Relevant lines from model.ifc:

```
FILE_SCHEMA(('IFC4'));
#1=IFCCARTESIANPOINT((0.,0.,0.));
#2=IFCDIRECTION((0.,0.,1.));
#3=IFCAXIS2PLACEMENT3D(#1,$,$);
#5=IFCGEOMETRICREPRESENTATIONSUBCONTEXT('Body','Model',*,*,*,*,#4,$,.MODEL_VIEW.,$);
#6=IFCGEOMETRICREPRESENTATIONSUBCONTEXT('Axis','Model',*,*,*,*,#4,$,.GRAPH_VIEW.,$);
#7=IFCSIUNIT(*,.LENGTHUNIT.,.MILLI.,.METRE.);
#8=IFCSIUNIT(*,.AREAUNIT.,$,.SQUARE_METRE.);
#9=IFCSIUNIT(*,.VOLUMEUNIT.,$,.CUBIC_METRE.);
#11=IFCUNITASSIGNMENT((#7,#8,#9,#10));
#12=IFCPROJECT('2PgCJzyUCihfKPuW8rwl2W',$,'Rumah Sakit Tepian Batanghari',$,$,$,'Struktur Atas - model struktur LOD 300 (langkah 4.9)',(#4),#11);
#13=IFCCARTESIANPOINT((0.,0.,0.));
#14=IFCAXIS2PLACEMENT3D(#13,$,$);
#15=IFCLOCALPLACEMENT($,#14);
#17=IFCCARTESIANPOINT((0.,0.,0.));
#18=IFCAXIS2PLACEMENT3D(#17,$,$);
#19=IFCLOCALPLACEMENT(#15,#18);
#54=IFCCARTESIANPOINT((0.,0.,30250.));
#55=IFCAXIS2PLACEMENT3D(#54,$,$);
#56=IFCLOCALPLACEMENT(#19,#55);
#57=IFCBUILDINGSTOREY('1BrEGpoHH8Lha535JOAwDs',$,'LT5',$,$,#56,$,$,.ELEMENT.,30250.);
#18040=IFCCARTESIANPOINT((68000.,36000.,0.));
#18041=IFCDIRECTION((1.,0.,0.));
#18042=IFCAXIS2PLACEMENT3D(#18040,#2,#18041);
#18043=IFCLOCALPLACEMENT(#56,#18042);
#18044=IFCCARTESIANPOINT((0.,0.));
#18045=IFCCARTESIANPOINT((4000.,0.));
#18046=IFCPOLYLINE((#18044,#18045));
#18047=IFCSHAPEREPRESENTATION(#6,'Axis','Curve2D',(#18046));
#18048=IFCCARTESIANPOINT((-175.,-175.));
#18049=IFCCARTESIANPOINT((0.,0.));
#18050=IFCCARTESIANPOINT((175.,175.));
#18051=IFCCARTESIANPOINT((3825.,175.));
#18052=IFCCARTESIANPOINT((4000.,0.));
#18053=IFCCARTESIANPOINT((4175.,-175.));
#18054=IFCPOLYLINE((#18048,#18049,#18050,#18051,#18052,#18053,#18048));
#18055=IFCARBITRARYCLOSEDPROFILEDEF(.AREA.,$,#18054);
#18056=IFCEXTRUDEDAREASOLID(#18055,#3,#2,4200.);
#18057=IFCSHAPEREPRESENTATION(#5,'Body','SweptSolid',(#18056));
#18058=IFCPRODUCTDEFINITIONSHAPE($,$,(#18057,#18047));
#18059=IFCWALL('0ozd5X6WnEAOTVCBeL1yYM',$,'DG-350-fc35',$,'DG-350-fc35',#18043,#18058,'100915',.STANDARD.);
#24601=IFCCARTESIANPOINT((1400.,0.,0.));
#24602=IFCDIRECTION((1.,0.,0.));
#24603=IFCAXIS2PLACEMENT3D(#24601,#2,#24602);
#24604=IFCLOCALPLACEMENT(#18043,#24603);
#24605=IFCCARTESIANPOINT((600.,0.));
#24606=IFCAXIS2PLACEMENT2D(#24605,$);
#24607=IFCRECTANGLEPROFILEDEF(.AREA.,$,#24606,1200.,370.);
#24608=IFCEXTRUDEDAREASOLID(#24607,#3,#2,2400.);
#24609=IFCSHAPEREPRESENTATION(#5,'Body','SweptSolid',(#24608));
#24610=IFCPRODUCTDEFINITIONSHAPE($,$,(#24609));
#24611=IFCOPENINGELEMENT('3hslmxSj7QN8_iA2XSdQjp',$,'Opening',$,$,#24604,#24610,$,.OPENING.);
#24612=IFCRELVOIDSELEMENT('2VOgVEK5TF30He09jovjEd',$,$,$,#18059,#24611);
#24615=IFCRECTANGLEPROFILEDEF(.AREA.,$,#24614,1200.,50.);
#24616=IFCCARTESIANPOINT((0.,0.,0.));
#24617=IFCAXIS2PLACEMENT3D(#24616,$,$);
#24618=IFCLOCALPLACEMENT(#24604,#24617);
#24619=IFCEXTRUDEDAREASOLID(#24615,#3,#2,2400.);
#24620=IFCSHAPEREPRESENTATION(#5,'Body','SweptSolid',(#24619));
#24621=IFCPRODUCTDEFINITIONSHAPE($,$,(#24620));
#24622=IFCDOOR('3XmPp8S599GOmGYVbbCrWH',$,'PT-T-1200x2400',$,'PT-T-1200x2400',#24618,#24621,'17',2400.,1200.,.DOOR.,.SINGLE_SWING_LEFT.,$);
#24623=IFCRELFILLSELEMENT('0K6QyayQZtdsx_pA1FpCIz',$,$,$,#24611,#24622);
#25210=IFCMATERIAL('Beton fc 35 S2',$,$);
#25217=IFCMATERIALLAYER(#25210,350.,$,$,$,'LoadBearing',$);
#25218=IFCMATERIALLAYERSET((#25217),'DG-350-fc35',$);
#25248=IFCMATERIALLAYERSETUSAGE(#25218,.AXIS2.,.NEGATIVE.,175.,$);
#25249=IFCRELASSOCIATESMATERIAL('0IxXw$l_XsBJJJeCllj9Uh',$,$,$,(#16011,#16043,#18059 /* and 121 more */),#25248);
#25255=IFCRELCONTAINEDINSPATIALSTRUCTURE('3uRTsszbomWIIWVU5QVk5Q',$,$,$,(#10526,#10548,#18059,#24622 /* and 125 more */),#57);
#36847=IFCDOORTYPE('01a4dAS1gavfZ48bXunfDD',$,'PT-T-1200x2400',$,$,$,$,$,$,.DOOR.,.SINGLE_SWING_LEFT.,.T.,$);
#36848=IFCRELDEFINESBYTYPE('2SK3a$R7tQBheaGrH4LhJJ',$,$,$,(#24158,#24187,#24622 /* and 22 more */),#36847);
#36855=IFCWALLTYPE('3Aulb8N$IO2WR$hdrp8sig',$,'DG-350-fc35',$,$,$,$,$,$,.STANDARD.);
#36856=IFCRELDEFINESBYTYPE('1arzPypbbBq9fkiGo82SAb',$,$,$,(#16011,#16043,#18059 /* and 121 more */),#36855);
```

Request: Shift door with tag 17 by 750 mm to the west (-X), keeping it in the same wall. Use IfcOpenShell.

```python
import ifcopenshell
import ifcopenshell.api.geometry
import ifcopenshell.util.placement
import ifcopenshell.util.unit

model = ifcopenshell.open("model.ifc")
unit_scale = ifcopenshell.util.unit.calculate_unit_scale(model)

door = model.by_id(24622)
opening = door.FillsVoids[0].RelatingOpeningElement
wall = opening.VoidsElements[0].RelatingBuildingElement

wall_matrix = ifcopenshell.util.placement.get_local_placement(wall.ObjectPlacement)
shift = wall_matrix[:3, 0] * -0.75 / unit_scale
before = ifcopenshell.util.placement.get_local_placement(door.ObjectPlacement)[:3, 3].copy()

# The door is placed relative to its opening, so it follows when the opening moves.
matrix = ifcopenshell.util.placement.get_local_placement(opening.ObjectPlacement)
matrix[:3, 3] += shift
ifcopenshell.api.geometry.edit_object_placement(
    model, product=opening, matrix=matrix, is_si=False, should_transform_children=True
)

after = ifcopenshell.util.placement.get_local_placement(door.ObjectPlacement)[:3, 3]
print("door moved by", (after - before).round(3) + 0.0)

model.write("model_rev.ifc")
```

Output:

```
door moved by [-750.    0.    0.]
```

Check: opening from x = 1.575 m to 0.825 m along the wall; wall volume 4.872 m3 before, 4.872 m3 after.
